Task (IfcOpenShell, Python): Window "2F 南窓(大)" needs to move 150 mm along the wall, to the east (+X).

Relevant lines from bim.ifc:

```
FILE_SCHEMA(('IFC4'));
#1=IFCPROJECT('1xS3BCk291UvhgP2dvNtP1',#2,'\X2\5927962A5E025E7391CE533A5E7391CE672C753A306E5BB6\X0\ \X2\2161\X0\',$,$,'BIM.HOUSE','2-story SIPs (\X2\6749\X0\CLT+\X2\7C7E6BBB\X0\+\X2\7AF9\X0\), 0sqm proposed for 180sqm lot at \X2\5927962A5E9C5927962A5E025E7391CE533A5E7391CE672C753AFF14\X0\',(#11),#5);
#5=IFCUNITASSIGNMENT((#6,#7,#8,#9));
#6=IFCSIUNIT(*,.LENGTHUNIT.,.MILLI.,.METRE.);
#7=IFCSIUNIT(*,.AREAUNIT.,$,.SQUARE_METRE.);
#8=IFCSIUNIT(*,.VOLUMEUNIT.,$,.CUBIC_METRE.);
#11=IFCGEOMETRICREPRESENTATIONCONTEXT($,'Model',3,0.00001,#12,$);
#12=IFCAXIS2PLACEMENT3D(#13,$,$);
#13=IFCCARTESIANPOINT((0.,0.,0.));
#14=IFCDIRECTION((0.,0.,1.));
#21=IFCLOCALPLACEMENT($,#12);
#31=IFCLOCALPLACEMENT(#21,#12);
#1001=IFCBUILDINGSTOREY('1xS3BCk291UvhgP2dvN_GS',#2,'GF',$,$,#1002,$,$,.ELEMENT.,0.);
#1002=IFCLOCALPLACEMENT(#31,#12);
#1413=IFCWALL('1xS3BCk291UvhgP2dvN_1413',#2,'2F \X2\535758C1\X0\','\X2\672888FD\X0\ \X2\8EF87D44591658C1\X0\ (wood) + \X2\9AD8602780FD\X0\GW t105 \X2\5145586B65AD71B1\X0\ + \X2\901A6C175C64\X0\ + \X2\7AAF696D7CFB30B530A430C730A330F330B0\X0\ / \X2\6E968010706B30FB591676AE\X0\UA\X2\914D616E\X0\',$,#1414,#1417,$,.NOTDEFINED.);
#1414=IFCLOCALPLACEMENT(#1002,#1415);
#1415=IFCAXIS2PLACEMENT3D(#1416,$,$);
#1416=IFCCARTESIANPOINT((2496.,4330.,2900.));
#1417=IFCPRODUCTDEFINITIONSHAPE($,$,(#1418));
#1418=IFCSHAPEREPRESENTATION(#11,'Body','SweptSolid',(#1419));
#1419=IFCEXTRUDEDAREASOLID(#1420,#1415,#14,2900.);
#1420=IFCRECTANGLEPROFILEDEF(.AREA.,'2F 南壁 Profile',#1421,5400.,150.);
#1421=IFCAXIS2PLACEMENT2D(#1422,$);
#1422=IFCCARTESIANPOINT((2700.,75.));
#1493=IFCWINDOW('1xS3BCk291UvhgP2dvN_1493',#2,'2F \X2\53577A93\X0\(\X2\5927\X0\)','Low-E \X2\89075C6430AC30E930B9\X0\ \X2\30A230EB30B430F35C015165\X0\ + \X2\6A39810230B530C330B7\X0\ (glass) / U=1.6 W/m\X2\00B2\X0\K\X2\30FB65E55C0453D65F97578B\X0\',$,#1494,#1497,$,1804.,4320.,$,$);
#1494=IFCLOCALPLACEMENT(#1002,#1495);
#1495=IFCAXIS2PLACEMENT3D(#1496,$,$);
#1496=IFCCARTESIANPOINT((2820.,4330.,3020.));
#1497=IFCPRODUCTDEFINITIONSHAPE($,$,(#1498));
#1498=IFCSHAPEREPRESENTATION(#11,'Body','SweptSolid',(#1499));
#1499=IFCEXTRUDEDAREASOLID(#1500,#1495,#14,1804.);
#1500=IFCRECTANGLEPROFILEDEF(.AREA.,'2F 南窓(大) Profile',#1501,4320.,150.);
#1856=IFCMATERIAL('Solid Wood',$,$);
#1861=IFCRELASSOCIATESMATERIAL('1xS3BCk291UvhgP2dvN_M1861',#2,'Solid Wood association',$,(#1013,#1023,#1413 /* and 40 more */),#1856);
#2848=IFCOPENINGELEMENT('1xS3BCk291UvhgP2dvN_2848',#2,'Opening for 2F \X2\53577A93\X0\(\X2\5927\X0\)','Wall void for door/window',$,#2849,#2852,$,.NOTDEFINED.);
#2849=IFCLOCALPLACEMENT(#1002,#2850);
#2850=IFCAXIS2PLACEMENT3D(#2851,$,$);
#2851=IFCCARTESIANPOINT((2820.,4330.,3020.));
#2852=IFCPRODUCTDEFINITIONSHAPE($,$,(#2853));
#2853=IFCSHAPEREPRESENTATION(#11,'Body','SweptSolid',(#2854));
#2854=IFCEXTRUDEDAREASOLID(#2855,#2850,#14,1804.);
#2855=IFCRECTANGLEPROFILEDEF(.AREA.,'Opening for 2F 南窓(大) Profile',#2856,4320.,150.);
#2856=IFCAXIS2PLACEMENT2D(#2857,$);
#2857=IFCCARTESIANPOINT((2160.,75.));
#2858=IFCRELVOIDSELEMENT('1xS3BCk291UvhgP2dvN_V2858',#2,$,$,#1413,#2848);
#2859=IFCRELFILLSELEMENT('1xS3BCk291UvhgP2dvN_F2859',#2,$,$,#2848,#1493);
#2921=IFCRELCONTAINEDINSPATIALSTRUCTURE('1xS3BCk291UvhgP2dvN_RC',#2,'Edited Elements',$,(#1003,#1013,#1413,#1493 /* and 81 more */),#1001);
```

```python
import ifcopenshell
import ifcopenshell.api.geometry
import ifcopenshell.util.placement
import ifcopenshell.util.unit

model = ifcopenshell.open("bim.ifc")
unit_scale = ifcopenshell.util.unit.calculate_unit_scale(model)

window = model.by_guid("1xS3BCk291UvhgP2dvN_1493")
opening = window.FillsVoids[0].RelatingOpeningElement
wall = opening.VoidsElements[0].RelatingBuildingElement

wall_matrix = ifcopenshell.util.placement.get_local_placement(wall.ObjectPlacement)
shift = wall_matrix[:3, 0] * 0.15 / unit_scale
before = ifcopenshell.util.placement.get_local_placement(window.ObjectPlacement)[:3, 3].copy()

# The window is not placed relative to its opening, so move both.
for product in (opening, window):
    matrix = ifcopenshell.util.placement.get_local_placement(product.ObjectPlacement)
    matrix[:3, 3] += shift
    ifcopenshell.api.geometry.edit_object_placement(model, product=product, matrix=matrix, is_si=False)

after = ifcopenshell.util.placement.get_local_placement(window.ObjectPlacement)[:3, 3]
print("window moved by", (after - before).round(3) + 0.0)

model.write("bim-out.ifc")
```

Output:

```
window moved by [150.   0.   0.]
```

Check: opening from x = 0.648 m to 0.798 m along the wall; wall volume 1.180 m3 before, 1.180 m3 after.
